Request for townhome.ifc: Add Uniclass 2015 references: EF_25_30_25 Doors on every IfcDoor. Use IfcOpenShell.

First a look at what the model holds.

```python
import ifcopenshell

model = ifcopenshell.open("townhome.ifc")
print(model.schema)
print("classifications:", [c.Name for c in model.by_type("IfcClassification")])
for ifc_class in ("IfcDoor", "IfcRoof", "IfcStair", "IfcWall", "IfcWindow"):
    print(ifc_class, len(model.by_type(ifc_class)))
```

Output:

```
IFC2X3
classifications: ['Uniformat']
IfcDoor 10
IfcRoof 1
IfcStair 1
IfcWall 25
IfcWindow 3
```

```python
import ifcopenshell
import ifcopenshell.api.classification

model = ifcopenshell.open("townhome.ifc")

# IFC2X3 requires Source and Edition and has no link from the project to the system.
system = model.create_entity("IfcClassification", Source="NBS", Edition="2015", Name="Uniclass 2015")

codes = {
    "IfcDoor": ("EF_25_30_25", "Doors"),
}
for ifc_class, (code, name) in codes.items():
    products = model.by_type(ifc_class)
    ifcopenshell.api.classification.add_reference(
        model, products=products, classification=system, identification=code, name=name
    )
    print(code, len(products))

model.write("townhome-out.ifc")
```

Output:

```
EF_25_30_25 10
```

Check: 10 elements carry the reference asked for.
